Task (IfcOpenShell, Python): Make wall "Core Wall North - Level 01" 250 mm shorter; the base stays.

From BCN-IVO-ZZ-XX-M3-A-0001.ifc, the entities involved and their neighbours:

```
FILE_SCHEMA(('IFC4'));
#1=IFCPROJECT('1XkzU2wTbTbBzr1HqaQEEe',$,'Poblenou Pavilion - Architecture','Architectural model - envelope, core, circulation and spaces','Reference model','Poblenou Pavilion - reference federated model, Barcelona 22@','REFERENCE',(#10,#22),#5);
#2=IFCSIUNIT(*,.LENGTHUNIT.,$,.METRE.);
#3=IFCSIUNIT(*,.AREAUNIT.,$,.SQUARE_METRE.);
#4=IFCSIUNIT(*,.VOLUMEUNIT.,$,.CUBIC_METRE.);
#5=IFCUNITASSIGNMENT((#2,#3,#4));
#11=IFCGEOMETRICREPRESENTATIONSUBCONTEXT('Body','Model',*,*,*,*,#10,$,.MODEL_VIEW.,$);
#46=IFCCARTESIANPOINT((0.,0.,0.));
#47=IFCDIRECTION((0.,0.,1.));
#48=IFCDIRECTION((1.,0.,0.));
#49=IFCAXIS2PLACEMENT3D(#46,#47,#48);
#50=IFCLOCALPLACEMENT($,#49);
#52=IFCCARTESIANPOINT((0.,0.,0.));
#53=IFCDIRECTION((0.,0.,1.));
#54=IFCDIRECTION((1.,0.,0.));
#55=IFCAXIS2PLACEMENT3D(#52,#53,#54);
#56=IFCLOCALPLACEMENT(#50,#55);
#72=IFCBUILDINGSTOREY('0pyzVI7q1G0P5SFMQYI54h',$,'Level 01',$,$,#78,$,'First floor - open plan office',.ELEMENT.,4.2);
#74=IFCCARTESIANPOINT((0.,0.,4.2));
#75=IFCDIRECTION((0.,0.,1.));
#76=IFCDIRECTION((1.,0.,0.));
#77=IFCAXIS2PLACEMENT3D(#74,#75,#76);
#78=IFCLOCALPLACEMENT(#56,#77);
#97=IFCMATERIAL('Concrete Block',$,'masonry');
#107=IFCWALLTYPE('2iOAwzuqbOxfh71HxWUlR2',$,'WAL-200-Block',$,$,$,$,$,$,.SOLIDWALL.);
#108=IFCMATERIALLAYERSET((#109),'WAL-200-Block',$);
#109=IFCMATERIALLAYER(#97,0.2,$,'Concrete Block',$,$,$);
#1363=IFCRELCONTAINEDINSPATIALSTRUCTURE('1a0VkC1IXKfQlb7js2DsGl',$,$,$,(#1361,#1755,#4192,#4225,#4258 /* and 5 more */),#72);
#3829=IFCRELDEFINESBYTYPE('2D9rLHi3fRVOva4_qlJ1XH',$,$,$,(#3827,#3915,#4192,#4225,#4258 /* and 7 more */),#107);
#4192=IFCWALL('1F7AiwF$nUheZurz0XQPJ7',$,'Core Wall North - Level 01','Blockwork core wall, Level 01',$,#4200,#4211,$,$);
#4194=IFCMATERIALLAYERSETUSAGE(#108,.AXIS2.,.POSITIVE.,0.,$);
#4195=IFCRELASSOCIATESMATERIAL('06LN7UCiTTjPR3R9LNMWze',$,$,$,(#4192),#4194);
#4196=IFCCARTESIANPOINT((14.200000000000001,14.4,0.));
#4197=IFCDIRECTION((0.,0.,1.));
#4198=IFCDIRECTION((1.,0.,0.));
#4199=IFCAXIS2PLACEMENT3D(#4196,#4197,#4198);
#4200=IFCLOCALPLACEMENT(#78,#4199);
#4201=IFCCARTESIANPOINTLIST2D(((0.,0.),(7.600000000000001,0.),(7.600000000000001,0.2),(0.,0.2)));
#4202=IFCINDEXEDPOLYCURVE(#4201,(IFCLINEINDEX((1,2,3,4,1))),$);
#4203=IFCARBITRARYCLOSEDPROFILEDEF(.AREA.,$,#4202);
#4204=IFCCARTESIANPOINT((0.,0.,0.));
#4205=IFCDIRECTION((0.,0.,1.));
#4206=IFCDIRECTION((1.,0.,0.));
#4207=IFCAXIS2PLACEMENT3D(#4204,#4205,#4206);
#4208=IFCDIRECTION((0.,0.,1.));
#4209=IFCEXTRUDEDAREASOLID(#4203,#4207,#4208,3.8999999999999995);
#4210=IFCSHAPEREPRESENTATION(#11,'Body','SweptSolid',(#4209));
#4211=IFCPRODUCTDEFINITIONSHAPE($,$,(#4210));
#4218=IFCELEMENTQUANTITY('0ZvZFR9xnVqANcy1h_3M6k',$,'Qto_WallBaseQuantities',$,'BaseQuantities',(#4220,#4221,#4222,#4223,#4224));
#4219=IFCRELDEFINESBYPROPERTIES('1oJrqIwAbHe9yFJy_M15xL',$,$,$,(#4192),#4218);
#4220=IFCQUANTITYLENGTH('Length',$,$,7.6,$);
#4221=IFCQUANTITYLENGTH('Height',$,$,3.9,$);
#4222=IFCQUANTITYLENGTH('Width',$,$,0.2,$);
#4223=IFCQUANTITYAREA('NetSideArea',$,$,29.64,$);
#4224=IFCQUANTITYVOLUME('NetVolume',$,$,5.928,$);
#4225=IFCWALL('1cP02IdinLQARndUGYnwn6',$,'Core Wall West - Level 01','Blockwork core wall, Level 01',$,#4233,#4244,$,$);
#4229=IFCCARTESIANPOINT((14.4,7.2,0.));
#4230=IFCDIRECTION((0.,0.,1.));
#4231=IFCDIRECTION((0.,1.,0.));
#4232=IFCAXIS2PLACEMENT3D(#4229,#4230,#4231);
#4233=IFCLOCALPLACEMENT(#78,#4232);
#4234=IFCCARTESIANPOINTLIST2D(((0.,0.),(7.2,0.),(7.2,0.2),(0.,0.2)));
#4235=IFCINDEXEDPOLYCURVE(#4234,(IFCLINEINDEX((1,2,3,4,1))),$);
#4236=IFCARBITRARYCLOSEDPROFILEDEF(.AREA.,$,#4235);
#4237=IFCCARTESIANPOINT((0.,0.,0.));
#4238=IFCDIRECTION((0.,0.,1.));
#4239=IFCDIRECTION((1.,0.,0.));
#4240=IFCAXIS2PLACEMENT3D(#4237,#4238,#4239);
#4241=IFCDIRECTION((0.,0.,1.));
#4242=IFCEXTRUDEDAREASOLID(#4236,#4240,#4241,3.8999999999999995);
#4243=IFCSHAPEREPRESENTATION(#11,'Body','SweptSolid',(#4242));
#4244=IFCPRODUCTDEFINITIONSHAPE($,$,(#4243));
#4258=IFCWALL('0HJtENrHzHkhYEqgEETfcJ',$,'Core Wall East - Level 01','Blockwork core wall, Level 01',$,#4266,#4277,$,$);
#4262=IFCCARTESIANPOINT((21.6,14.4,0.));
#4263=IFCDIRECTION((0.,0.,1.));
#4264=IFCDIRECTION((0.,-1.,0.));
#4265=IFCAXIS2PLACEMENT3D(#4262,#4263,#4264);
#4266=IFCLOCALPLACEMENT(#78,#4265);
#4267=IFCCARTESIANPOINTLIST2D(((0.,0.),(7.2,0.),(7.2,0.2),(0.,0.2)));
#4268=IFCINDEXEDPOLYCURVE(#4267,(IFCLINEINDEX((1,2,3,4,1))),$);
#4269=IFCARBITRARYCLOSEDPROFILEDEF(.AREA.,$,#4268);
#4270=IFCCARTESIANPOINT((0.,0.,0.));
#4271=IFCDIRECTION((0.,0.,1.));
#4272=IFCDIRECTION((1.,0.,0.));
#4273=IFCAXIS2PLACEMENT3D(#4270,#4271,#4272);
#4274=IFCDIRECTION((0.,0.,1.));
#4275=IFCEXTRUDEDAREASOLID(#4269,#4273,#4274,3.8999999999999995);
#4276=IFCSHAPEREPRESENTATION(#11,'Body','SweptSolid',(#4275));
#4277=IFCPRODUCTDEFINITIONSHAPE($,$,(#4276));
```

```python
import ifcopenshell
import ifcopenshell.api.pset
import ifcopenshell.geom
import ifcopenshell.util.element
import ifcopenshell.util.representation
import ifcopenshell.util.shape
import ifcopenshell.util.unit

model = ifcopenshell.open("BCN-IVO-ZZ-XX-M3-A-0001.ifc")
unit_scale = ifcopenshell.util.unit.calculate_unit_scale(model)
area_scale = ifcopenshell.util.unit.calculate_unit_scale(model, "AREAUNIT")
volume_scale = ifcopenshell.util.unit.calculate_unit_scale(model, "VOLUMEUNIT")
settings = ifcopenshell.geom.settings()


def volume(element):
    """Net volume in cubic metres, openings subtracted."""
    shape = ifcopenshell.geom.create_shape(settings, element)
    return ifcopenshell.util.shape.get_volume(shape.geometry)


wall = model.by_guid("1F7AiwF$nUheZurz0XQPJ7")
before = volume(wall)

body = ifcopenshell.util.representation.get_representation(wall, "Model", "Body")
solid = body.Items[0]
old_height = solid.Depth
solid.Depth -= 0.25 / unit_scale
after = volume(wall)
thickness = 0.2  # wall thickness in metres

# Update the stored height, areas and volumes.
qto = model.by_id(ifcopenshell.util.element.get_pset(wall, "Qto_WallBaseQuantities", should_inherit=False)["id"])
ifcopenshell.api.pset.edit_qto(model, qto=qto, properties={
    "Height": solid.Depth,
    "NetSideArea": after / thickness / area_scale,
    "NetVolume": after / volume_scale,
})

print(f"height {old_height:g} -> {solid.Depth:g}, volume {before:.3f} -> {after:.3f} m3")

model.write("BCN-IVO-ZZ-XX-M3-A-0001_updated.ifc")
```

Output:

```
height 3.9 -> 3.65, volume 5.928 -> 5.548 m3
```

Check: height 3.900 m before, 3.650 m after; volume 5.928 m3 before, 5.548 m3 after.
